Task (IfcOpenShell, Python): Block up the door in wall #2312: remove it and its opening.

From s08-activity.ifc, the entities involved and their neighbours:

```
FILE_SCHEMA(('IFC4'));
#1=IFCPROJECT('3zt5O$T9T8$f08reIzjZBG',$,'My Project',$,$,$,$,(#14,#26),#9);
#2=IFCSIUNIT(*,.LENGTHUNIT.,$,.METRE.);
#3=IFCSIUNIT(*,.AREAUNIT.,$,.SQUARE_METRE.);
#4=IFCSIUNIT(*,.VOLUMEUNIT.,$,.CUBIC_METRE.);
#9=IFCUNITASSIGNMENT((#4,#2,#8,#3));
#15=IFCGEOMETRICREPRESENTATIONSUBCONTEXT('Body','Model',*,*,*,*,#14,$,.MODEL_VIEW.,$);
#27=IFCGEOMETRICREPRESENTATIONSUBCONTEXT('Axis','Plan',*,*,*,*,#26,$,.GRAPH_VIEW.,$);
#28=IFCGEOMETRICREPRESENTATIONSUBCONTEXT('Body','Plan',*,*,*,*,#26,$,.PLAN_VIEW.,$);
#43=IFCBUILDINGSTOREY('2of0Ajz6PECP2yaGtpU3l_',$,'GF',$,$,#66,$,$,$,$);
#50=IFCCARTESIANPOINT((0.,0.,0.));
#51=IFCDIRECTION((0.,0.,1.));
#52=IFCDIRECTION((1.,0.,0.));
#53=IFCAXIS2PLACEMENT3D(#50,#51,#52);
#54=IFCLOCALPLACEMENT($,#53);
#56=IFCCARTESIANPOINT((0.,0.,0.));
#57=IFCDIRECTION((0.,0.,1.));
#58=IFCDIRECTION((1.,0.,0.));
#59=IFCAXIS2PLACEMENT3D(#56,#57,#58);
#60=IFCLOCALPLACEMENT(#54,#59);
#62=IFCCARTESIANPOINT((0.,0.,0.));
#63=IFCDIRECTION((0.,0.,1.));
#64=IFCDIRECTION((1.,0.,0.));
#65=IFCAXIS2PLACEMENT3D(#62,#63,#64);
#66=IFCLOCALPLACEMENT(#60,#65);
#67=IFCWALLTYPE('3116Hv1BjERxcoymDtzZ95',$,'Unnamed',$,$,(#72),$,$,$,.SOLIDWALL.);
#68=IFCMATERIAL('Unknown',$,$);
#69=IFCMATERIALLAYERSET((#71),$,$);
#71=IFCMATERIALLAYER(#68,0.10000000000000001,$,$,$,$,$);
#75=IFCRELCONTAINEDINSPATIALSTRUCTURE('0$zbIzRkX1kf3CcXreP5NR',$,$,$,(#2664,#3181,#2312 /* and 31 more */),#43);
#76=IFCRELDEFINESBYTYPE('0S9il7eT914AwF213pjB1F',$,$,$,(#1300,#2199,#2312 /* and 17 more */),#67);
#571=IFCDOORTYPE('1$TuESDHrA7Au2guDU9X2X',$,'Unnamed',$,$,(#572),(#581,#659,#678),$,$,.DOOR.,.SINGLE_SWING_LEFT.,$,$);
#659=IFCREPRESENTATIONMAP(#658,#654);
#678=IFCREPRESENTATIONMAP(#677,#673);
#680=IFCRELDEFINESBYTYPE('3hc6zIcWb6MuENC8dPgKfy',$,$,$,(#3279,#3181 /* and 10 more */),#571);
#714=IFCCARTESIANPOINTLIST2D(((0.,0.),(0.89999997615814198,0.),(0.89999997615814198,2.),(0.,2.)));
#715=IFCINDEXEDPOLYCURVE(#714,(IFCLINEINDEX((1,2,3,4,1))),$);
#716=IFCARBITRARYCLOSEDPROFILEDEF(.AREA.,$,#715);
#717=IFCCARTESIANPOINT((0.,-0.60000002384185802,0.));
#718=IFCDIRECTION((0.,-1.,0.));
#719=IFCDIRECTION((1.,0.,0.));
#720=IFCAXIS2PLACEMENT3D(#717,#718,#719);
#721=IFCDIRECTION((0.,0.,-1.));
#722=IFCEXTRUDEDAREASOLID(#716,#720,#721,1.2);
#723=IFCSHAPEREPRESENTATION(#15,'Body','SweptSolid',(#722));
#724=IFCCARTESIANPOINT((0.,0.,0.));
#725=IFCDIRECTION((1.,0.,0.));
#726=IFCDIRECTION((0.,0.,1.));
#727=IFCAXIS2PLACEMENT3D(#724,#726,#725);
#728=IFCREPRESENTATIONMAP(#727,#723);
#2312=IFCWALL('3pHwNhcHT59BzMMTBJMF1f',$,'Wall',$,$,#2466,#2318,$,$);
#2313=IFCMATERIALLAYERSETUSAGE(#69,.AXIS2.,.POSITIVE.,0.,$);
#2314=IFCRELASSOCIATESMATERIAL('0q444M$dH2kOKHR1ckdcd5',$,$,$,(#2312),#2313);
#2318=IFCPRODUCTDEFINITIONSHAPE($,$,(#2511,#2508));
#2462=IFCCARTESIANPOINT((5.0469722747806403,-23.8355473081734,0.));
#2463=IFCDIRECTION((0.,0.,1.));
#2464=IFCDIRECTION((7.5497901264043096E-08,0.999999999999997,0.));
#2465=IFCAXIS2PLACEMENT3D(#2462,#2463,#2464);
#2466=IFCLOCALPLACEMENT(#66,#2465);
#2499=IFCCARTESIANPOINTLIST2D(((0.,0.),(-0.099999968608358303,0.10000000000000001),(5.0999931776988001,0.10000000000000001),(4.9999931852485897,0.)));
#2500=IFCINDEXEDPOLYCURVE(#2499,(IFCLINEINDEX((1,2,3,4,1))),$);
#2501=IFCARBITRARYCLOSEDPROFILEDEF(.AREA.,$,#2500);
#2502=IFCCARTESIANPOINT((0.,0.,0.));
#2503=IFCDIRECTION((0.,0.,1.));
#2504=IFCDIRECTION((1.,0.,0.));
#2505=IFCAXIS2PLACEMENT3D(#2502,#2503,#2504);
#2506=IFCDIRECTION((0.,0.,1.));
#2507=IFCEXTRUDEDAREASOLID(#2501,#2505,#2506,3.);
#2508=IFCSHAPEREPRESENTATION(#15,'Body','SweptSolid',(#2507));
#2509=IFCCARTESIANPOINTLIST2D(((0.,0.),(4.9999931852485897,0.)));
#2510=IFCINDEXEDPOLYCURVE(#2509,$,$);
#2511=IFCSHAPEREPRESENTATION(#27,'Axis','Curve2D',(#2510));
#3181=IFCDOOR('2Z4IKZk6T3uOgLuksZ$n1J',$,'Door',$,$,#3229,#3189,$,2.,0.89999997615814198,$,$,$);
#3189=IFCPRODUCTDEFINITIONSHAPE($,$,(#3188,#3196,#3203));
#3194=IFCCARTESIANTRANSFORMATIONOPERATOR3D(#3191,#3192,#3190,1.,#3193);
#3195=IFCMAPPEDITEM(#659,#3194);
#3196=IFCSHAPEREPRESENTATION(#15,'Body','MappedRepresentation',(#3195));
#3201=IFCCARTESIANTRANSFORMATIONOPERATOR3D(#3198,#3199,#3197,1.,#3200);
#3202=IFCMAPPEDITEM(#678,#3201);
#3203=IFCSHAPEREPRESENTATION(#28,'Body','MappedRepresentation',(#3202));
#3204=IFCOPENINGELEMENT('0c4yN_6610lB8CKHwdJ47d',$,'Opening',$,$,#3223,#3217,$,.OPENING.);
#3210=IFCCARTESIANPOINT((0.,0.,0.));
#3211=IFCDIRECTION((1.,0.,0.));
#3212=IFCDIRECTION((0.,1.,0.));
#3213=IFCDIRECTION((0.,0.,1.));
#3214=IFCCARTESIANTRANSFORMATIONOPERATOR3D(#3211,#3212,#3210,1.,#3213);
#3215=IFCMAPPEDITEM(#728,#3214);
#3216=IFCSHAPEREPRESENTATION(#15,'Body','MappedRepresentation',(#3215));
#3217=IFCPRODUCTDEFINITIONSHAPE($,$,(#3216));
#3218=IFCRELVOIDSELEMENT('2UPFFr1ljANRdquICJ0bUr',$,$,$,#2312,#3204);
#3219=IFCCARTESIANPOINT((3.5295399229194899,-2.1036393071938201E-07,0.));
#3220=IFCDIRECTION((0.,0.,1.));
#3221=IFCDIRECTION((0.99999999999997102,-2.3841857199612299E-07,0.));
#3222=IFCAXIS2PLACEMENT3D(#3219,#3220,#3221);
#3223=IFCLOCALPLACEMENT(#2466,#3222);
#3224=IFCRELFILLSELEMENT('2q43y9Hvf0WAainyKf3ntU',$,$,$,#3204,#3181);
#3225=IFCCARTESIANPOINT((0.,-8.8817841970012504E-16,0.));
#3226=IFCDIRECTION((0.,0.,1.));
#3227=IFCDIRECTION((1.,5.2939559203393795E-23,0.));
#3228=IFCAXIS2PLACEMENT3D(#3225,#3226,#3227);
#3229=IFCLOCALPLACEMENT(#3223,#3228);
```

```python
import ifcopenshell
import ifcopenshell.api.feature
import ifcopenshell.api.root
import ifcopenshell.geom
import ifcopenshell.util.shape

model = ifcopenshell.open("s08-activity.ifc")
settings = ifcopenshell.geom.settings()


def volume(element):
    """Net volume in cubic metres, openings subtracted."""
    shape = ifcopenshell.geom.create_shape(settings, element)
    return ifcopenshell.util.shape.get_volume(shape.geometry)


door = model.by_guid("2Z4IKZk6T3uOgLuksZ$n1J")
opening = door.FillsVoids[0].RelatingOpeningElement
wall = opening.VoidsElements[0].RelatingBuildingElement
before = volume(wall)

ifcopenshell.api.root.remove_product(model, product=door)
ifcopenshell.api.feature.remove_feature(model, feature=opening)

after = volume(wall)

print(f"wall volume {before:.3f} -> {after:.3f} m3")

model.write("s08-activity_updated.ifc")
```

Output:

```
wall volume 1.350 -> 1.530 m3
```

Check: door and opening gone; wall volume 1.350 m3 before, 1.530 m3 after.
